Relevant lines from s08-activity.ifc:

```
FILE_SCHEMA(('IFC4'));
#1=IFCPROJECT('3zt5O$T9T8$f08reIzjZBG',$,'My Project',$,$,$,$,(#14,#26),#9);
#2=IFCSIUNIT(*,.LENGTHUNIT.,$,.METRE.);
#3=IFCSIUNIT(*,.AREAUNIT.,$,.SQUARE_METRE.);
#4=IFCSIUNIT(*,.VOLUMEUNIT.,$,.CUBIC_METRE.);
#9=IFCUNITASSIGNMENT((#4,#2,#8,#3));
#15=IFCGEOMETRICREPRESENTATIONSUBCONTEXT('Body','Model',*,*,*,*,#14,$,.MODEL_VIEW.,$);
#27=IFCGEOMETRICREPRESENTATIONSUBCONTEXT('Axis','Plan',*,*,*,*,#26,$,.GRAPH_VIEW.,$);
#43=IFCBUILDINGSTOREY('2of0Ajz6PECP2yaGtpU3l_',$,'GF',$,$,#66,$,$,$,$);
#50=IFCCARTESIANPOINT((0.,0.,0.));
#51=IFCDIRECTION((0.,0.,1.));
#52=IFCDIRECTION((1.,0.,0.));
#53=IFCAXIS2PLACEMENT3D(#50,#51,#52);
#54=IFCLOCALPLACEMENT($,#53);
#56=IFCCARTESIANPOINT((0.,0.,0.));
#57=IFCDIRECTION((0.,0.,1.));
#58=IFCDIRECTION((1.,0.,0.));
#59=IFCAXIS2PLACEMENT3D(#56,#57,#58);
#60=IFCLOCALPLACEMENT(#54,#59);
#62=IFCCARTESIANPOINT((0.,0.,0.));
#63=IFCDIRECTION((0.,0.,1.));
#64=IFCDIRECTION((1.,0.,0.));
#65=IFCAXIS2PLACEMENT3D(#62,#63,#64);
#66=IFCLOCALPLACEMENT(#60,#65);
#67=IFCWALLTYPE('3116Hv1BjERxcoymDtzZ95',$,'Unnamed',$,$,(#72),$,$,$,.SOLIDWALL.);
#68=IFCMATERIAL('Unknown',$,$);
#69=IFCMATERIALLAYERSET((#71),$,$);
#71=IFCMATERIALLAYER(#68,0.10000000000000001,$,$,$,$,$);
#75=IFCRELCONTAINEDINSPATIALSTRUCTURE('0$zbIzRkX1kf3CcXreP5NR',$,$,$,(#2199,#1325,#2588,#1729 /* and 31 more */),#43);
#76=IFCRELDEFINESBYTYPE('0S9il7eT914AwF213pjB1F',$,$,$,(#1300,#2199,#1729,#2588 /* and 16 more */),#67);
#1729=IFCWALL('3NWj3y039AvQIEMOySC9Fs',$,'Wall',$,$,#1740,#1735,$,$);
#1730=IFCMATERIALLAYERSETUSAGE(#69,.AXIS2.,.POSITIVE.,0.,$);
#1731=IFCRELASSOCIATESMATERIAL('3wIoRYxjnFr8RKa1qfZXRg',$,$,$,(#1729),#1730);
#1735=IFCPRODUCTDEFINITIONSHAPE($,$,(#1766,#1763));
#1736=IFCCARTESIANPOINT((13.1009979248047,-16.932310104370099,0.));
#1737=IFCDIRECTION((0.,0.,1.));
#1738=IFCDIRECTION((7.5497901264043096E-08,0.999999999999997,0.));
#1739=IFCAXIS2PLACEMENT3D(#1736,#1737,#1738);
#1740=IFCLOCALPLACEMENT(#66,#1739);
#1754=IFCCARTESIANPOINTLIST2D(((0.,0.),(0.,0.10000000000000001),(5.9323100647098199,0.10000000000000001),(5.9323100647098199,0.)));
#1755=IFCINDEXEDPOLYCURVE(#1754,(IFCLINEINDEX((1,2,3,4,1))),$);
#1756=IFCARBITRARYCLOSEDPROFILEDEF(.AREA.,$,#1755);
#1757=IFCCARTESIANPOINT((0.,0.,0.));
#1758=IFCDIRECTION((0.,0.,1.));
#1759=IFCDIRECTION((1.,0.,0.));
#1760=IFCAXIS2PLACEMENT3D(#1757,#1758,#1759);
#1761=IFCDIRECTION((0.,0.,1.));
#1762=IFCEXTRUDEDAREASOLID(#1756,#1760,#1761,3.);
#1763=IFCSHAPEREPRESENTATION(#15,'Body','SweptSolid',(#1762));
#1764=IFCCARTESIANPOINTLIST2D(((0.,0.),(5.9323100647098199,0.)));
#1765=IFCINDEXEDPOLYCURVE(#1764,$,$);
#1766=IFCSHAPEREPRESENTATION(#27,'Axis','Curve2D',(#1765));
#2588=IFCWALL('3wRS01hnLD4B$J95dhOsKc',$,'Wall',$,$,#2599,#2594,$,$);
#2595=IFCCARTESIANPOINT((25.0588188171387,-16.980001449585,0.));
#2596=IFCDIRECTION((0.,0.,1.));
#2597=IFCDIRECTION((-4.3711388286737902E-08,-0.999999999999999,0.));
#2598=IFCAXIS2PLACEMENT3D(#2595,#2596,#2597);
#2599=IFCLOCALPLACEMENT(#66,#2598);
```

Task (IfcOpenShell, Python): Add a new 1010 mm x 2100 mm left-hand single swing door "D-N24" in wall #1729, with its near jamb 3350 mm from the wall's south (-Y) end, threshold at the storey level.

```python
import numpy as np
import ifcopenshell
import ifcopenshell.api.feature
import ifcopenshell.api.geometry
import ifcopenshell.api.root
import ifcopenshell.api.spatial
import ifcopenshell.geom
import ifcopenshell.util.element
import ifcopenshell.util.placement
import ifcopenshell.util.representation
import ifcopenshell.util.shape
import ifcopenshell.util.unit

model = ifcopenshell.open("s08-activity.ifc")
unit_scale = ifcopenshell.util.unit.calculate_unit_scale(model)
settings = ifcopenshell.geom.settings()


def volume(element):
    """Net volume in cubic metres, openings subtracted."""
    shape = ifcopenshell.geom.create_shape(settings, element)
    return ifcopenshell.util.shape.get_volume(shape.geometry)


wall = model.by_guid("3NWj3y039AvQIEMOySC9Fs")
storey = ifcopenshell.util.element.get_container(wall, ifc_class="IfcBuildingStorey")
context = ifcopenshell.util.representation.get_context(model, "Model", "Body", "MODEL_VIEW")
before = volume(wall)

width, height, from_end, sill = 1.01, 2.1, 3.35, 0.0  # metres

# The wall runs along its own X axis, and the end named is its -X end.
wall_shape = ifcopenshell.geom.create_shape(settings, wall)
x, y, z = ifcopenshell.util.shape.get_vertices(wall_shape.geometry).T
start = x.min() + from_end
face, thickness = float(y.min()), float(y.max() - y.min())
wall_matrix = ifcopenshell.util.placement.get_local_placement(wall.ObjectPlacement)
level = ifcopenshell.util.placement.get_local_placement(storey.ObjectPlacement)[2, 3]


def in_wall(x, y):
    """Placement at x, y metres in the wall's axes, at sill height."""
    matrix = wall_matrix.copy()
    matrix[:, 3] = wall_matrix @ np.array([x / unit_scale, y / unit_scale, 0.0, 1.0])
    matrix[2, 3] = level + sill / unit_scale
    return matrix


# Opening: a box that overshoots both wall faces by 50 mm.
opening = ifcopenshell.api.root.create_entity(model, ifc_class="IfcOpeningElement", predefined_type="OPENING")
box = ifcopenshell.api.geometry.add_wall_representation(
    model, context=context, length=width, height=height, thickness=thickness + 0.1
)
ifcopenshell.api.geometry.assign_representation(model, product=opening, representation=box)
ifcopenshell.api.geometry.edit_object_placement(model, product=opening, matrix=in_wall(start, face - 0.05), is_si=False)
ifcopenshell.api.feature.add_feature(model, feature=opening, element=wall)

door = ifcopenshell.api.root.create_entity(model, ifc_class="IfcDoor", name="D-N24", predefined_type="DOOR")
door.OverallWidth, door.OverallHeight = width / unit_scale, height / unit_scale
door.OperationType = "SINGLE_SWING_LEFT"
body = ifcopenshell.api.geometry.add_door_representation(
    model,
    context=context,
    overall_width=door.OverallWidth,
    overall_height=door.OverallHeight,
    operation_type="SINGLE_SWING_LEFT",
    lining_properties={"LiningDepth": thickness / unit_scale, "ThresholdDepth": thickness / unit_scale},
)
ifcopenshell.api.geometry.assign_representation(model, product=door, representation=body)
ifcopenshell.api.spatial.assign_container(model, products=[door], relating_structure=storey)
ifcopenshell.api.feature.add_filling(model, opening=opening, element=door)

# The lining spans the wall, so the door starts at the wall face.
ifcopenshell.api.geometry.edit_object_placement(model, product=door, matrix=in_wall(start, face), is_si=False)

after = volume(wall)

print(f"wall volume {before:.3f} -> {after:.3f} m3")

model.write("s08-activity_edited.ifc")
```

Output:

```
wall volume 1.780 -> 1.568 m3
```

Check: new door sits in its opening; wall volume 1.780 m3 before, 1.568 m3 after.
